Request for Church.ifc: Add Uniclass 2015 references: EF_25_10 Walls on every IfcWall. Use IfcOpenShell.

First a look at what the model holds.

```python
import ifcopenshell

model = ifcopenshell.open("Church.ifc")
print(model.schema)
print("classifications:", [c.Name for c in model.by_type("IfcClassification")])
for ifc_class in ("IfcDoor", "IfcRoof", "IfcStair", "IfcWall", "IfcWindow"):
    print(ifc_class, len(model.by_type(ifc_class)))
```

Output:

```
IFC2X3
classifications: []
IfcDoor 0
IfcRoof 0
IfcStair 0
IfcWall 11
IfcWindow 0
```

```python
import ifcopenshell
import ifcopenshell.api.classification

model = ifcopenshell.open("Church.ifc")

# IFC2X3 requires Source and Edition and has no link from the project to the system.
system = model.create_entity("IfcClassification", Source="NBS", Edition="2015", Name="Uniclass 2015")

codes = {
    "IfcWall": ("EF_25_10", "Walls"),
}
for ifc_class, (code, name) in codes.items():
    products = model.by_type(ifc_class)
    ifcopenshell.api.classification.add_reference(
        model, products=products, classification=system, identification=code, name=name
    )
    print(code, len(products))

model.write("Church_edited.ifc")
```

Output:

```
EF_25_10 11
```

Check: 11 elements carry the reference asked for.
